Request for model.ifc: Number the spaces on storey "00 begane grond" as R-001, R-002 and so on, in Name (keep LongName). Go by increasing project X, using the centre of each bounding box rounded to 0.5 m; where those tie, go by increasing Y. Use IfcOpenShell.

First a look at what the model holds.

```python
import ifcopenshell
import ifcopenshell.util.element
import ifcopenshell.util.placement

model = ifcopenshell.open("model.ifc")
print(model.schema)
storey = next(s for s in model.by_type("IfcBuildingStorey") if s.Name == "00 begane grond")
spaces = [e for e in ifcopenshell.util.element.get_decomposition(storey) if e.is_a("IfcSpace")]
for e in sorted(spaces, key=lambda e: e.id()):
    origin = ifcopenshell.util.placement.get_local_placement(e.ObjectPlacement)[:3, 3]
    print(e.id(), e.Name, e.LongName, origin.round(2) + 0.0, sep=" | ")
```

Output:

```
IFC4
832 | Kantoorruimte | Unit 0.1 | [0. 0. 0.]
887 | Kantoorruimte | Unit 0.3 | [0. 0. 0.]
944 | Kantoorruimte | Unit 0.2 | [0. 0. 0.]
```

```python
import ifcopenshell
import ifcopenshell.geom
import ifcopenshell.util.element
import ifcopenshell.util.shape

model = ifcopenshell.open("model.ifc")
settings = ifcopenshell.geom.settings()
settings.set("use-world-coords", True)


def centre(element):
    shape = ifcopenshell.geom.create_shape(settings, element)
    return ifcopenshell.util.shape.get_bbox_centroid(shape.geometry)


storey = next(s for s in model.by_type("IfcBuildingStorey") if s.Name == "00 begane grond")
spaces = [e for e in ifcopenshell.util.element.get_decomposition(storey) if e.is_a("IfcSpace")]

# Insertion points can sit at a corner or the storey origin, so sort by the geometry (in metres).
centres = {e: centre(e) for e in spaces}
spaces.sort(key=lambda e: (round(centres[e][0] / 0.5), centres[e][1]))

for i, e in enumerate(spaces, start=1):
    number = f"R-0{i:02d}"
    e.Name = number
    print(e.id(), number)

model.write("model_rev.ifc")
```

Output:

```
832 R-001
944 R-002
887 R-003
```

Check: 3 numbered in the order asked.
